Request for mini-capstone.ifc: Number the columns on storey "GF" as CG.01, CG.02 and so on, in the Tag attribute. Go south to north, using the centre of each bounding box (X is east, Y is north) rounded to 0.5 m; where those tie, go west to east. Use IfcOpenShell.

First a look at what the model holds.

```python
import ifcopenshell
import ifcopenshell.util.element
import ifcopenshell.util.placement

model = ifcopenshell.open("mini-capstone.ifc")
print(model.schema)
storey = next(s for s in model.by_type("IfcBuildingStorey") if s.Name == "GF")
columns = [e for e in ifcopenshell.util.element.get_decomposition(storey) if e.is_a("IfcColumn")]
for e in sorted(columns, key=lambda e: e.id()):
    origin = ifcopenshell.util.placement.get_local_placement(e.ObjectPlacement)[:3, 3]
    print(e.id(), e.Tag, e.Name, origin.round(2) + 0.0, sep=" | ")
```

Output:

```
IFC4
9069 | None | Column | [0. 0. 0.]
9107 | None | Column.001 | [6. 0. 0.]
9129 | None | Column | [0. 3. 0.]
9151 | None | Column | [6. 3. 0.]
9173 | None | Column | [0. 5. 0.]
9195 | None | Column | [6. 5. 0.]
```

```python
import ifcopenshell
import ifcopenshell.geom
import ifcopenshell.util.element
import ifcopenshell.util.shape

model = ifcopenshell.open("mini-capstone.ifc")
settings = ifcopenshell.geom.settings()
settings.set("use-world-coords", True)


def centre(element):
    shape = ifcopenshell.geom.create_shape(settings, element)
    return ifcopenshell.util.shape.get_bbox_centroid(shape.geometry)


storey = next(s for s in model.by_type("IfcBuildingStorey") if s.Name == "GF")
columns = [e for e in ifcopenshell.util.element.get_decomposition(storey) if e.is_a("IfcColumn")]

# Insertion points can sit at a corner or the storey origin, so sort by the geometry (in metres).
centres = {e: centre(e) for e in columns}
columns.sort(key=lambda e: (round(centres[e][1] / 0.5), centres[e][0]))

for i, e in enumerate(columns, start=1):
    number = f"CG.{i:02d}"
    e.Tag = number
    print(e.id(), number)

model.write("mini-capstone_edited.ifc")
```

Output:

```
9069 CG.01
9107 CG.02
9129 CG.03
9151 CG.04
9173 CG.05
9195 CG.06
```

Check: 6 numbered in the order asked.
